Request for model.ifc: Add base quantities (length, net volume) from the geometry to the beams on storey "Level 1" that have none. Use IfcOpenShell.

First a look at what the model holds.

```python
import ifcopenshell
import ifcopenshell.util.element
import ifcopenshell.util.unit

model = ifcopenshell.open("model.ifc")
print(model.schema)
for unit_type in ("LENGTHUNIT", "AREAUNIT", "VOLUMEUNIT"):
    print(unit_type, ifcopenshell.util.unit.calculate_unit_scale(model, unit_type))
storey = next(s for s in model.by_type("IfcBuildingStorey") if s.Name == "Level 1")
beams = [e for e in ifcopenshell.util.element.get_decomposition(storey) if e.is_a("IfcBeam")]
for e in sorted(beams, key=lambda e: e.id()):
    print(e.id(), e.is_a(), e.Name, list(ifcopenshell.util.element.get_psets(e, qtos_only=True)), sep=" | ")
```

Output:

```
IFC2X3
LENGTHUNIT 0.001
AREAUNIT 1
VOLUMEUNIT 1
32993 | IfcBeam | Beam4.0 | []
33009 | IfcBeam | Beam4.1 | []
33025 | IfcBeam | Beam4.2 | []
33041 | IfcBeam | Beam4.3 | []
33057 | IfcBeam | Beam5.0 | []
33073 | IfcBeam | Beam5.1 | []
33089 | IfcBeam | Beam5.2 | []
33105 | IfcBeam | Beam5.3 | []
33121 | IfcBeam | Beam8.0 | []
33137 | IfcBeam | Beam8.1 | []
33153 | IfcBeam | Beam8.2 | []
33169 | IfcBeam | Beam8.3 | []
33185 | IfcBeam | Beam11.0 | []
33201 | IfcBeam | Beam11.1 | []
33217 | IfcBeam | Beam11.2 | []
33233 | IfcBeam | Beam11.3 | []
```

```python
import ifcopenshell
import ifcopenshell.api.pset
import ifcopenshell.geom
import ifcopenshell.util.element
import ifcopenshell.util.shape
import ifcopenshell.util.unit

model = ifcopenshell.open("model.ifc")
unit_scale = ifcopenshell.util.unit.calculate_unit_scale(model)
volume_scale = ifcopenshell.util.unit.calculate_unit_scale(model, "VOLUMEUNIT")
settings = ifcopenshell.geom.settings()

storey = next(s for s in model.by_type("IfcBuildingStorey") if s.Name == "Level 1")
beams = [e for e in ifcopenshell.util.element.get_decomposition(storey) if e.is_a("IfcBeam")]

for e in sorted(beams, key=lambda e: e.id()):
    if ifcopenshell.util.element.get_psets(e, qtos_only=True, should_inherit=False):
        continue
    # Geometry comes back in metres, in the element's own axes.
    shape = ifcopenshell.geom.create_shape(settings, e)
    values = {
        "Length": ifcopenshell.util.shape.get_max_xyz(shape.geometry) / unit_scale,
        "NetVolume": ifcopenshell.util.shape.get_volume(shape.geometry) / volume_scale,
    }
    qto = ifcopenshell.api.pset.add_qto(model, product=e, name="BaseQuantities")
    ifcopenshell.api.pset.edit_qto(model, qto=qto, properties=values)
    print(e.id(), {k: round(v, 3) for k, v in values.items()})

model.write("model_rev.ifc")
```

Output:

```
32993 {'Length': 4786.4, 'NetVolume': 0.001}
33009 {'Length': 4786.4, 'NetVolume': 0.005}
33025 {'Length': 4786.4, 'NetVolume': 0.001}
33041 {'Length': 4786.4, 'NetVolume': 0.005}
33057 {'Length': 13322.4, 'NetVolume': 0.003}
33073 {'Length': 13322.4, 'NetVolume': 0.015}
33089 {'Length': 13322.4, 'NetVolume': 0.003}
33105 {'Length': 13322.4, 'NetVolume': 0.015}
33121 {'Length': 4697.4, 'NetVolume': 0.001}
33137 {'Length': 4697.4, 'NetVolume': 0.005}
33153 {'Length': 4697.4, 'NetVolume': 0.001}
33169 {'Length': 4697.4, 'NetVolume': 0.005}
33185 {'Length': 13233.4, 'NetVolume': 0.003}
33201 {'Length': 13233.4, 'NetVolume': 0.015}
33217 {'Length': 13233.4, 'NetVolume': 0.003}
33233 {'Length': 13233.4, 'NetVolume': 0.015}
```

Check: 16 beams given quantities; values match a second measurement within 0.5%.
